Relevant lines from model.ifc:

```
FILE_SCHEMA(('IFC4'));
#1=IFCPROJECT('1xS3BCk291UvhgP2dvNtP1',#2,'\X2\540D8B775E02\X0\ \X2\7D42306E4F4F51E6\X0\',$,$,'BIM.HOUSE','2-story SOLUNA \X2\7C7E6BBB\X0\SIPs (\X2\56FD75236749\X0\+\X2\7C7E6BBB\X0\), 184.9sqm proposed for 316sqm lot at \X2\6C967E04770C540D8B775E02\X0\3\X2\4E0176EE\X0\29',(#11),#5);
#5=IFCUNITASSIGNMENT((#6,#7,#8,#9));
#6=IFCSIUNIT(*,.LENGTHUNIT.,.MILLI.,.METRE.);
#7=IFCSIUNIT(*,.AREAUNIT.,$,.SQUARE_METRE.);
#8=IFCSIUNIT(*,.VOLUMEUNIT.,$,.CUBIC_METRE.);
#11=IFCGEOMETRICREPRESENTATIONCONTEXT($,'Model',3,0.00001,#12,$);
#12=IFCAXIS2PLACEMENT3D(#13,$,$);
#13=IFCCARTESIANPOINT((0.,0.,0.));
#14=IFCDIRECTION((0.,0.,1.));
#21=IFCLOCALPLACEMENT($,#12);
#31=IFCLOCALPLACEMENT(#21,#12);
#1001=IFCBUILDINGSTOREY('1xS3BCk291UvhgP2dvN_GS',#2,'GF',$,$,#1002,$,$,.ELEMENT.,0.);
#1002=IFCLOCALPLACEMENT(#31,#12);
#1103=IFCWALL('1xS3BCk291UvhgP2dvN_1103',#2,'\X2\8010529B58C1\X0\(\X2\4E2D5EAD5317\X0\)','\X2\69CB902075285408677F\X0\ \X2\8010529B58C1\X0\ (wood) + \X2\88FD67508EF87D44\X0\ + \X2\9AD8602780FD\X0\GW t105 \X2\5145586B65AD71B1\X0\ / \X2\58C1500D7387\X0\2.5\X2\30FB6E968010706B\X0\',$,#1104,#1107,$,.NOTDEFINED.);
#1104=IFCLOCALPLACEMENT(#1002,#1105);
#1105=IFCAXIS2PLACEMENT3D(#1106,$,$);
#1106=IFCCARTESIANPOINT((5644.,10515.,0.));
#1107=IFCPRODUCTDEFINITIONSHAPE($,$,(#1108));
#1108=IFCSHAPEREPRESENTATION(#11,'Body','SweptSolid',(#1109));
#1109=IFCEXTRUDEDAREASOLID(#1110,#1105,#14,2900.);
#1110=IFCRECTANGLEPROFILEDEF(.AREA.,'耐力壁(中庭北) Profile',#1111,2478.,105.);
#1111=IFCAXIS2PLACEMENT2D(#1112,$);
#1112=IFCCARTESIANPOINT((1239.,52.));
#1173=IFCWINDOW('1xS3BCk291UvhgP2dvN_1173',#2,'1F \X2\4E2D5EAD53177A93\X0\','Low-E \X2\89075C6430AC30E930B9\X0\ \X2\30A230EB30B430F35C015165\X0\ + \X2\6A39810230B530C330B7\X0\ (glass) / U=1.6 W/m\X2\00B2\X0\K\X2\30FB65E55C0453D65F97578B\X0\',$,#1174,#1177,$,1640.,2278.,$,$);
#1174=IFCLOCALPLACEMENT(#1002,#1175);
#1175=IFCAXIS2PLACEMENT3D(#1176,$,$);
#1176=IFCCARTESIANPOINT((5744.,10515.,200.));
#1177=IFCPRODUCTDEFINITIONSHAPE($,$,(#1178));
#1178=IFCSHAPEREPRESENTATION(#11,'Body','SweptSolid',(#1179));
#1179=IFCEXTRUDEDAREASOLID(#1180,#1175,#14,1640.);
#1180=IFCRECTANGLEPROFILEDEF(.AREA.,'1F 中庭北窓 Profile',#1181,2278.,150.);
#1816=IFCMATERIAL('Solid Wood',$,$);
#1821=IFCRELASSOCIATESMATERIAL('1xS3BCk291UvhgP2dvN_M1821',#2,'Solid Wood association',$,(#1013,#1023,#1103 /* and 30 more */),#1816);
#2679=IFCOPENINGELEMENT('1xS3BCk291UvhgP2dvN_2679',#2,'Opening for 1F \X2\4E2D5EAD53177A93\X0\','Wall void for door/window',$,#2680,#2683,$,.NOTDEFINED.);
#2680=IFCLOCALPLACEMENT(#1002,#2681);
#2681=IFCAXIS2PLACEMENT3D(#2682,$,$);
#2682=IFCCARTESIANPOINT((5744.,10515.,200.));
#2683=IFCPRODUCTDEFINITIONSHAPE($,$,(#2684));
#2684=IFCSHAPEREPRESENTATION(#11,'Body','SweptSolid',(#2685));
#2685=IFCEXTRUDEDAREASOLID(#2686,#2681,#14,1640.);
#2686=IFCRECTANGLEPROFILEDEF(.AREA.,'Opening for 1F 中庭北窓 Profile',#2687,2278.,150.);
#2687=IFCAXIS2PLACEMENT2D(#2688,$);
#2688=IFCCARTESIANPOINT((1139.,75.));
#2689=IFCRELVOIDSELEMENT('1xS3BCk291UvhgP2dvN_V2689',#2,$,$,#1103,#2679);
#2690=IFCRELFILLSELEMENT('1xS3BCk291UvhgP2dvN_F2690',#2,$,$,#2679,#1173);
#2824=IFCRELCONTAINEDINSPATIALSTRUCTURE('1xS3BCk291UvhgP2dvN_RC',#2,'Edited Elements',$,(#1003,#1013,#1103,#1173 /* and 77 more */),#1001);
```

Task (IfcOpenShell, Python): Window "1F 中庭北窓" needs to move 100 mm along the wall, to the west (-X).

```python
import ifcopenshell
import ifcopenshell.api.geometry
import ifcopenshell.util.placement

model = ifcopenshell.open("model.ifc")

window = model.by_id(1173)
opening = window.FillsVoids[0].RelatingOpeningElement
wall = opening.VoidsElements[0].RelatingBuildingElement

wall_matrix = ifcopenshell.util.placement.get_local_placement(wall.ObjectPlacement)
shift = wall_matrix[:3, 0] * -100.0
before = ifcopenshell.util.placement.get_local_placement(window.ObjectPlacement)[:3, 3].copy()

# The window is not placed relative to its opening, so move both.
for product in (opening, window):
    matrix = ifcopenshell.util.placement.get_local_placement(product.ObjectPlacement)
    matrix[:3, 3] += shift
    ifcopenshell.api.geometry.edit_object_placement(model, product=product, matrix=matrix, is_si=False)

after = ifcopenshell.util.placement.get_local_placement(window.ObjectPlacement)[:3, 3]
print("window moved by", (after - before).round(3) + 0.0)

model.write("model_updated.ifc")
```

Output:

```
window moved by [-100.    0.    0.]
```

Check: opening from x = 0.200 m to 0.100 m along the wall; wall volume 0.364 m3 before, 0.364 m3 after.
